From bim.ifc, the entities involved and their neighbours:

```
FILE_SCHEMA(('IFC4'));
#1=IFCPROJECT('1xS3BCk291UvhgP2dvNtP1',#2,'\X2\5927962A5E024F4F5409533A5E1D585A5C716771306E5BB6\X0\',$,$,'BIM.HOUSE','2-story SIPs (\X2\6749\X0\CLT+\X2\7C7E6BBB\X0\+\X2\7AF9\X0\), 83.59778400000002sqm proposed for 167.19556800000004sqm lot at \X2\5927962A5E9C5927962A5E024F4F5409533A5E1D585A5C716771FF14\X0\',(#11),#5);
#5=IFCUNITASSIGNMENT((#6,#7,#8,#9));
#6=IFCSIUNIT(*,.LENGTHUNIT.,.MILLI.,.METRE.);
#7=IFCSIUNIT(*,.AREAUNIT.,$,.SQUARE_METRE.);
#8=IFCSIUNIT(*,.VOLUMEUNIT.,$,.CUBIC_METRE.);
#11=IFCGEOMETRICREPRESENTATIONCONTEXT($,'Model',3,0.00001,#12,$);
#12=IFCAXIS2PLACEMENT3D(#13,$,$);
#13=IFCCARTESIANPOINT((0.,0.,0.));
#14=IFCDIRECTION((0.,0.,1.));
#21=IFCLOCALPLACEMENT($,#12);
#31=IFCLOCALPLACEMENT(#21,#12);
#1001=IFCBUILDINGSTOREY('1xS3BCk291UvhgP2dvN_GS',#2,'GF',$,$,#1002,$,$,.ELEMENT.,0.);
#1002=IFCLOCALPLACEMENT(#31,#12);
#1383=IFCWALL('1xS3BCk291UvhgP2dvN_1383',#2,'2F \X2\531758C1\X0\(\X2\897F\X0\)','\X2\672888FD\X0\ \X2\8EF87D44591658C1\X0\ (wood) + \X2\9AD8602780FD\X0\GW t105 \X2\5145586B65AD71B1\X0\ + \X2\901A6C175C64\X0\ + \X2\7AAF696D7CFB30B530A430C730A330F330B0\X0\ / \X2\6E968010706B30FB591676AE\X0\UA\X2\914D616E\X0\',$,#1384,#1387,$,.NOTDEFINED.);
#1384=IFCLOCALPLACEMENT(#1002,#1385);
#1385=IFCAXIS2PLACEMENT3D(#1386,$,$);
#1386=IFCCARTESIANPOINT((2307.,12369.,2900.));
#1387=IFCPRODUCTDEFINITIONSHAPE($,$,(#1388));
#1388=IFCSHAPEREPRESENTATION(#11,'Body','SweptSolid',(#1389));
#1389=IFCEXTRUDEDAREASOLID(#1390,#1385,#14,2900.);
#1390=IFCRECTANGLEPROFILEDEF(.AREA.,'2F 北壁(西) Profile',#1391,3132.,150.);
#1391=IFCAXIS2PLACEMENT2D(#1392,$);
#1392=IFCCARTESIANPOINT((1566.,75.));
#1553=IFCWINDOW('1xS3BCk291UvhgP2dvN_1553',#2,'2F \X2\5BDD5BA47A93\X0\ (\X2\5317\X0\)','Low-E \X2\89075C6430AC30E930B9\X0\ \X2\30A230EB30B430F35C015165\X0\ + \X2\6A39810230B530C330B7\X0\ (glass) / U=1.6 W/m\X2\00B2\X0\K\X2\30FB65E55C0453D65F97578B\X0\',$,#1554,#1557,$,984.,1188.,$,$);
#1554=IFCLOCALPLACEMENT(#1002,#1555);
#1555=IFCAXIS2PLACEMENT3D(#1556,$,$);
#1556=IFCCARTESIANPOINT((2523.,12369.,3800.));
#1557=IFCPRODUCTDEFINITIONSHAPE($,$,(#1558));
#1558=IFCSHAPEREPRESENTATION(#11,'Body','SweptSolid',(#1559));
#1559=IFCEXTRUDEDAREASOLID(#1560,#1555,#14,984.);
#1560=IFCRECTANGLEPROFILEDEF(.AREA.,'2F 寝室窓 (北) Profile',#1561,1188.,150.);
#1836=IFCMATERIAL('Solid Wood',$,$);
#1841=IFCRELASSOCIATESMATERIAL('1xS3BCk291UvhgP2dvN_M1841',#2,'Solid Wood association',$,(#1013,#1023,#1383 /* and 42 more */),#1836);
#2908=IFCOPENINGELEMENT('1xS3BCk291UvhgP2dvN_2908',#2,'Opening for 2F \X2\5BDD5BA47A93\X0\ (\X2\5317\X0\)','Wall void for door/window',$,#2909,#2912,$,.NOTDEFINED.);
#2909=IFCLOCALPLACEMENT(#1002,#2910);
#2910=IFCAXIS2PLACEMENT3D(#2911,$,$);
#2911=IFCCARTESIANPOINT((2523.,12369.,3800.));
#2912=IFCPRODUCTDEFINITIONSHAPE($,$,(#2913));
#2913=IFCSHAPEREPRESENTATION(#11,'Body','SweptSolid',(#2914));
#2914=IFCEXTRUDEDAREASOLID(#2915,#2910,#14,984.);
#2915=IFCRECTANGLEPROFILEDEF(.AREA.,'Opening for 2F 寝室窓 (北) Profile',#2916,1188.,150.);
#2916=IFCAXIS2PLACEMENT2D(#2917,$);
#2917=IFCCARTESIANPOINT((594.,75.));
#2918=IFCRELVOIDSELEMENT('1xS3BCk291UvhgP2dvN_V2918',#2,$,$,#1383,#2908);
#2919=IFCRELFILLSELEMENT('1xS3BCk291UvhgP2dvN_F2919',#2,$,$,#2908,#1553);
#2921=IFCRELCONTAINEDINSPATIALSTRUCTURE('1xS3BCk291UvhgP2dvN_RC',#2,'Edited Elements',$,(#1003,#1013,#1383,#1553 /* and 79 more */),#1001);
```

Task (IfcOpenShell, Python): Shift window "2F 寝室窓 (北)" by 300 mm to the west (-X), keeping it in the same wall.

```python
import ifcopenshell
import ifcopenshell.api.geometry
import ifcopenshell.util.placement
import ifcopenshell.util.unit

model = ifcopenshell.open("bim.ifc")
unit_scale = ifcopenshell.util.unit.calculate_unit_scale(model)

window = model.by_guid("1xS3BCk291UvhgP2dvN_1553")
opening = window.FillsVoids[0].RelatingOpeningElement
wall = opening.VoidsElements[0].RelatingBuildingElement

wall_matrix = ifcopenshell.util.placement.get_local_placement(wall.ObjectPlacement)
shift = wall_matrix[:3, 0] * -0.3 / unit_scale
before = ifcopenshell.util.placement.get_local_placement(window.ObjectPlacement)[:3, 3].copy()

# The window is not placed relative to its opening, so move both.
for product in (opening, window):
    matrix = ifcopenshell.util.placement.get_local_placement(product.ObjectPlacement)
    matrix[:3, 3] += shift
    ifcopenshell.api.geometry.edit_object_placement(model, product=product, matrix=matrix, is_si=False)

after = ifcopenshell.util.placement.get_local_placement(window.ObjectPlacement)[:3, 3]
print("window moved by", (after - before).round(3) + 0.0)

model.write("bim_v2.ifc")
```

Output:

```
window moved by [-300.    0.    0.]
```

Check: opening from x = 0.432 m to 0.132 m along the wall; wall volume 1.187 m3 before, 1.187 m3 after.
